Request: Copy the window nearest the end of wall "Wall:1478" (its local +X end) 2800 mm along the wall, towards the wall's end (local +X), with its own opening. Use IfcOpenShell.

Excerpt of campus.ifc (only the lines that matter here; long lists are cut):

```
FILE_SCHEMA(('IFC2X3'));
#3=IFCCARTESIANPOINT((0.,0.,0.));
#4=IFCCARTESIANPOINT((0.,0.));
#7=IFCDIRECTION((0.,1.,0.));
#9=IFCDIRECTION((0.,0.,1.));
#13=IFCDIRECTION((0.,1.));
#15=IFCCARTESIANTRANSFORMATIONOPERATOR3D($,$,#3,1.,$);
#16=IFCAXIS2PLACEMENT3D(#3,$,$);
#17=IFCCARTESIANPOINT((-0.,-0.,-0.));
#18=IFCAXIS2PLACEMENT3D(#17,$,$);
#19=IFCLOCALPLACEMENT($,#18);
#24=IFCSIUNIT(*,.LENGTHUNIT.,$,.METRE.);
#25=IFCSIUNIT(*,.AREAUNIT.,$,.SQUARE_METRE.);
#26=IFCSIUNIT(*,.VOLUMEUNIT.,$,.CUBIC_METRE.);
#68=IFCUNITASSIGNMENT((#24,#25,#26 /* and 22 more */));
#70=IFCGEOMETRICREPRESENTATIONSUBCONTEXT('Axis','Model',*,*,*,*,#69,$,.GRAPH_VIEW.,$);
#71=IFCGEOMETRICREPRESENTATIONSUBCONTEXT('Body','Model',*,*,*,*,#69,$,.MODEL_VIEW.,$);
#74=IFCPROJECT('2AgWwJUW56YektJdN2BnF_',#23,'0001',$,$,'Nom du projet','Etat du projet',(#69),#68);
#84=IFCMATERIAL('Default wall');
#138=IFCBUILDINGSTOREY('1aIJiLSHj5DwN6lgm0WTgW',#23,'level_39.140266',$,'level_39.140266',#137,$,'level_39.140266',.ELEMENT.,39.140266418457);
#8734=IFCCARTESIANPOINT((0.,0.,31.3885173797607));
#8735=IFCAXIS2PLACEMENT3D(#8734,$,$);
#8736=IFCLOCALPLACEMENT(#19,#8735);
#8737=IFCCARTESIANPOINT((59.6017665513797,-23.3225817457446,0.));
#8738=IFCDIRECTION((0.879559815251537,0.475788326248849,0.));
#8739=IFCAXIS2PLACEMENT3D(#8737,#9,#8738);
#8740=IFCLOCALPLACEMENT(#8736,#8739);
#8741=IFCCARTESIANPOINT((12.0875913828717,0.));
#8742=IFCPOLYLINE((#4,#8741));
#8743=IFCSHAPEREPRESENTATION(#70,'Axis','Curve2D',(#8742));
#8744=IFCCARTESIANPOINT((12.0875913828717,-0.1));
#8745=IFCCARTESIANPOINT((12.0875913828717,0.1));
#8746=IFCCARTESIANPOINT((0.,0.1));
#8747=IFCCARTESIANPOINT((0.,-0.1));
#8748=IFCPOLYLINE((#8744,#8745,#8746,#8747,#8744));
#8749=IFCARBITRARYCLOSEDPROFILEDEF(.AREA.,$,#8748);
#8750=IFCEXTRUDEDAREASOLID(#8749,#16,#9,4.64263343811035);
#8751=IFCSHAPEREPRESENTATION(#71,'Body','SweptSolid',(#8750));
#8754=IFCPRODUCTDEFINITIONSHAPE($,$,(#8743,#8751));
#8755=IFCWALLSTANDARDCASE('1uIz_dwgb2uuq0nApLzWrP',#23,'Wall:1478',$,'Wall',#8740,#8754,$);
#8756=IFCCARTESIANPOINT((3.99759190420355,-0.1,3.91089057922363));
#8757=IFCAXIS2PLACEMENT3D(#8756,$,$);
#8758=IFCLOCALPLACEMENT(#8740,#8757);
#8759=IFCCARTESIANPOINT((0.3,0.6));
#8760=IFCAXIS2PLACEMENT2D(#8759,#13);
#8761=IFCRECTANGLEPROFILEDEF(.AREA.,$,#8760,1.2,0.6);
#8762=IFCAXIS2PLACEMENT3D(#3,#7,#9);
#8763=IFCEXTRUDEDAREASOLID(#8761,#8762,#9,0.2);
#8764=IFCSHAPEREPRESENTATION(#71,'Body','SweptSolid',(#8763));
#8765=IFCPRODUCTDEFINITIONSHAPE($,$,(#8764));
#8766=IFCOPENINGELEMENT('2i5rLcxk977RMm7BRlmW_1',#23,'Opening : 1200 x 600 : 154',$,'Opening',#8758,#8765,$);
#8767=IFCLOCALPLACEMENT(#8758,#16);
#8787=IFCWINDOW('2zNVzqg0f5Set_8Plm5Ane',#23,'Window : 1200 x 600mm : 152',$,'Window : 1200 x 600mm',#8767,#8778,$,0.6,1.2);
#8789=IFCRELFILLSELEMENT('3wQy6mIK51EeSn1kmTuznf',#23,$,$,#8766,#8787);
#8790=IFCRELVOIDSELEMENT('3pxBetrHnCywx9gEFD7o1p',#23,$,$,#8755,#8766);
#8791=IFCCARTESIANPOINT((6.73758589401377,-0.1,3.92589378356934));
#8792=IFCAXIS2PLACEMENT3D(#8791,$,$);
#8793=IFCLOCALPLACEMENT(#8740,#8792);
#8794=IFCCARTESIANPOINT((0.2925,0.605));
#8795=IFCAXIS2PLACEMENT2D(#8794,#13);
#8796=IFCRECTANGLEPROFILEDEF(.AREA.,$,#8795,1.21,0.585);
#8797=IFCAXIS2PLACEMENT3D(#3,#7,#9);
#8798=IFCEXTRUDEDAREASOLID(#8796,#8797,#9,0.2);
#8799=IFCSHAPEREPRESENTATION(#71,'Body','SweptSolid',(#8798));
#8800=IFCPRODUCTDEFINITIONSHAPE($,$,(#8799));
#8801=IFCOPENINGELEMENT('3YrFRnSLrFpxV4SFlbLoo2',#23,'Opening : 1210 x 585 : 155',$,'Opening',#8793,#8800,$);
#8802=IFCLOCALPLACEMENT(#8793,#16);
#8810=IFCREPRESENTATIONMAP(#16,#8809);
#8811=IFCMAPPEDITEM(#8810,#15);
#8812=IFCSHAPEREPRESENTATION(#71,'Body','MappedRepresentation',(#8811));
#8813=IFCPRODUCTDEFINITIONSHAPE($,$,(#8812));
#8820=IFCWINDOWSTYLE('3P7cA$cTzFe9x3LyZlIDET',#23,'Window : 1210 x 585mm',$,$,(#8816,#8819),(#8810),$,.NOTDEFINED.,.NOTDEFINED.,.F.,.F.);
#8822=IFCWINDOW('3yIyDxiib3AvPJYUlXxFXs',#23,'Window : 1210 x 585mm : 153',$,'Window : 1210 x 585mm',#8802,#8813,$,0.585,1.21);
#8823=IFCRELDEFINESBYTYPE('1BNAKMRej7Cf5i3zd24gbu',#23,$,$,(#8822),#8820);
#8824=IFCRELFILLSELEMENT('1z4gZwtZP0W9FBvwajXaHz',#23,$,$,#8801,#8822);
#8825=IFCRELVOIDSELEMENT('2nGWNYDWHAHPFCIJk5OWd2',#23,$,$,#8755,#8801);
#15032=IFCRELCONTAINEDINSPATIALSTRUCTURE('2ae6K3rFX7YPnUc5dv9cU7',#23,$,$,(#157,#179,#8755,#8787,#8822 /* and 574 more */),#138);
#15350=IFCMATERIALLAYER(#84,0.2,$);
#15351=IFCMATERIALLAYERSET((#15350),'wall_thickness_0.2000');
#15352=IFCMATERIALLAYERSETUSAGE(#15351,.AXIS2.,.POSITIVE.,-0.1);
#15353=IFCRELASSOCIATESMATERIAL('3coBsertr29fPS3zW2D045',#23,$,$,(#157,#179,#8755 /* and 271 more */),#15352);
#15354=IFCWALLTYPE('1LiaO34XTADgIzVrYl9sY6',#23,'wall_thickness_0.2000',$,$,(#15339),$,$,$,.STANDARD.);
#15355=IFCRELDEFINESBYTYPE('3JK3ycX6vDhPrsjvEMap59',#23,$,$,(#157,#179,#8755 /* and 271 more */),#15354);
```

```python
import ifcopenshell
import ifcopenshell.api.feature
import ifcopenshell.api.geometry
import ifcopenshell.api.root
import ifcopenshell.geom
import ifcopenshell.util.element
import ifcopenshell.util.placement
import ifcopenshell.util.shape

model = ifcopenshell.open("campus.ifc")
settings = ifcopenshell.geom.settings()


def volume(element):
    """Net volume in cubic metres, openings subtracted."""
    shape = ifcopenshell.geom.create_shape(settings, element)
    return ifcopenshell.util.shape.get_volume(shape.geometry)


window = model.by_guid("3yIyDxiib3AvPJYUlXxFXs")
opening = window.FillsVoids[0].RelatingOpeningElement
wall = opening.VoidsElements[0].RelatingBuildingElement
before = volume(wall)
shift = ifcopenshell.util.placement.get_local_placement(wall.ObjectPlacement)[:3, 0] * 2.8

# copy_class copies the void relationship, type, container and properties, but no geometry.
new_opening = ifcopenshell.api.root.copy_class(model, product=opening)
new_opening.Representation = ifcopenshell.util.element.copy_deep(
    model, opening.Representation, exclude=["IfcGeometricRepresentationContext", "IfcRepresentationMap"]
)
new_opening.Name = "Opening : 1210 x 585"
new_window = ifcopenshell.api.root.copy_class(model, product=window)
new_window.Representation = ifcopenshell.util.element.copy_deep(
    model, window.Representation, exclude=["IfcGeometricRepresentationContext", "IfcRepresentationMap"]
)
new_window.Name = "Window : 1210 x 585mm"
fills = ifcopenshell.api.feature.add_filling(model, opening=new_opening, element=new_window)
fills.OwnerHistory = new_window.OwnerHistory  # required in IFC2X3

for old, new in ((opening, new_opening), (window, new_window)):
    matrix = ifcopenshell.util.placement.get_local_placement(old.ObjectPlacement)
    matrix[:3, 3] += shift
    ifcopenshell.api.geometry.edit_object_placement(model, product=new, matrix=matrix, is_si=False)

after = volume(wall)

print(f"wall volume {before:.3f} -> {after:.3f} m3")

model.write("campus_edited.ifc")
```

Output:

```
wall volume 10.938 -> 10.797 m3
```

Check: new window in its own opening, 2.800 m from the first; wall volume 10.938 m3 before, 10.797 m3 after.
